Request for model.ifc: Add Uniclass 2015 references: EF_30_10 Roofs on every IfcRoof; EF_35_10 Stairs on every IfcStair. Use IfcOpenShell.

First a look at what the model holds.

```python
import ifcopenshell

model = ifcopenshell.open("model.ifc")
print(model.schema)
print("classifications:", [c.Name for c in model.by_type("IfcClassification")])
for ifc_class in ("IfcDoor", "IfcRoof", "IfcStair", "IfcWall", "IfcWindow"):
    print(ifc_class, len(model.by_type(ifc_class)))
```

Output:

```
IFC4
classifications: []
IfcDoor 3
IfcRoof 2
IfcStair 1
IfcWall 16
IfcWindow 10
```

```python
import ifcopenshell
import ifcopenshell.api.classification

model = ifcopenshell.open("model.ifc")

system = ifcopenshell.api.classification.add_classification(model, classification="Uniclass 2015")

codes = {
    "IfcRoof": ("EF_30_10", "Roofs"),
    "IfcStair": ("EF_35_10", "Stairs"),
}
for ifc_class, (code, name) in codes.items():
    products = model.by_type(ifc_class)
    ifcopenshell.api.classification.add_reference(
        model, products=products, classification=system, identification=code, name=name
    )
    print(code, len(products))

model.write("model_edited.ifc")
```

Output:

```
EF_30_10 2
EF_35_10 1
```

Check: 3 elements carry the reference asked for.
